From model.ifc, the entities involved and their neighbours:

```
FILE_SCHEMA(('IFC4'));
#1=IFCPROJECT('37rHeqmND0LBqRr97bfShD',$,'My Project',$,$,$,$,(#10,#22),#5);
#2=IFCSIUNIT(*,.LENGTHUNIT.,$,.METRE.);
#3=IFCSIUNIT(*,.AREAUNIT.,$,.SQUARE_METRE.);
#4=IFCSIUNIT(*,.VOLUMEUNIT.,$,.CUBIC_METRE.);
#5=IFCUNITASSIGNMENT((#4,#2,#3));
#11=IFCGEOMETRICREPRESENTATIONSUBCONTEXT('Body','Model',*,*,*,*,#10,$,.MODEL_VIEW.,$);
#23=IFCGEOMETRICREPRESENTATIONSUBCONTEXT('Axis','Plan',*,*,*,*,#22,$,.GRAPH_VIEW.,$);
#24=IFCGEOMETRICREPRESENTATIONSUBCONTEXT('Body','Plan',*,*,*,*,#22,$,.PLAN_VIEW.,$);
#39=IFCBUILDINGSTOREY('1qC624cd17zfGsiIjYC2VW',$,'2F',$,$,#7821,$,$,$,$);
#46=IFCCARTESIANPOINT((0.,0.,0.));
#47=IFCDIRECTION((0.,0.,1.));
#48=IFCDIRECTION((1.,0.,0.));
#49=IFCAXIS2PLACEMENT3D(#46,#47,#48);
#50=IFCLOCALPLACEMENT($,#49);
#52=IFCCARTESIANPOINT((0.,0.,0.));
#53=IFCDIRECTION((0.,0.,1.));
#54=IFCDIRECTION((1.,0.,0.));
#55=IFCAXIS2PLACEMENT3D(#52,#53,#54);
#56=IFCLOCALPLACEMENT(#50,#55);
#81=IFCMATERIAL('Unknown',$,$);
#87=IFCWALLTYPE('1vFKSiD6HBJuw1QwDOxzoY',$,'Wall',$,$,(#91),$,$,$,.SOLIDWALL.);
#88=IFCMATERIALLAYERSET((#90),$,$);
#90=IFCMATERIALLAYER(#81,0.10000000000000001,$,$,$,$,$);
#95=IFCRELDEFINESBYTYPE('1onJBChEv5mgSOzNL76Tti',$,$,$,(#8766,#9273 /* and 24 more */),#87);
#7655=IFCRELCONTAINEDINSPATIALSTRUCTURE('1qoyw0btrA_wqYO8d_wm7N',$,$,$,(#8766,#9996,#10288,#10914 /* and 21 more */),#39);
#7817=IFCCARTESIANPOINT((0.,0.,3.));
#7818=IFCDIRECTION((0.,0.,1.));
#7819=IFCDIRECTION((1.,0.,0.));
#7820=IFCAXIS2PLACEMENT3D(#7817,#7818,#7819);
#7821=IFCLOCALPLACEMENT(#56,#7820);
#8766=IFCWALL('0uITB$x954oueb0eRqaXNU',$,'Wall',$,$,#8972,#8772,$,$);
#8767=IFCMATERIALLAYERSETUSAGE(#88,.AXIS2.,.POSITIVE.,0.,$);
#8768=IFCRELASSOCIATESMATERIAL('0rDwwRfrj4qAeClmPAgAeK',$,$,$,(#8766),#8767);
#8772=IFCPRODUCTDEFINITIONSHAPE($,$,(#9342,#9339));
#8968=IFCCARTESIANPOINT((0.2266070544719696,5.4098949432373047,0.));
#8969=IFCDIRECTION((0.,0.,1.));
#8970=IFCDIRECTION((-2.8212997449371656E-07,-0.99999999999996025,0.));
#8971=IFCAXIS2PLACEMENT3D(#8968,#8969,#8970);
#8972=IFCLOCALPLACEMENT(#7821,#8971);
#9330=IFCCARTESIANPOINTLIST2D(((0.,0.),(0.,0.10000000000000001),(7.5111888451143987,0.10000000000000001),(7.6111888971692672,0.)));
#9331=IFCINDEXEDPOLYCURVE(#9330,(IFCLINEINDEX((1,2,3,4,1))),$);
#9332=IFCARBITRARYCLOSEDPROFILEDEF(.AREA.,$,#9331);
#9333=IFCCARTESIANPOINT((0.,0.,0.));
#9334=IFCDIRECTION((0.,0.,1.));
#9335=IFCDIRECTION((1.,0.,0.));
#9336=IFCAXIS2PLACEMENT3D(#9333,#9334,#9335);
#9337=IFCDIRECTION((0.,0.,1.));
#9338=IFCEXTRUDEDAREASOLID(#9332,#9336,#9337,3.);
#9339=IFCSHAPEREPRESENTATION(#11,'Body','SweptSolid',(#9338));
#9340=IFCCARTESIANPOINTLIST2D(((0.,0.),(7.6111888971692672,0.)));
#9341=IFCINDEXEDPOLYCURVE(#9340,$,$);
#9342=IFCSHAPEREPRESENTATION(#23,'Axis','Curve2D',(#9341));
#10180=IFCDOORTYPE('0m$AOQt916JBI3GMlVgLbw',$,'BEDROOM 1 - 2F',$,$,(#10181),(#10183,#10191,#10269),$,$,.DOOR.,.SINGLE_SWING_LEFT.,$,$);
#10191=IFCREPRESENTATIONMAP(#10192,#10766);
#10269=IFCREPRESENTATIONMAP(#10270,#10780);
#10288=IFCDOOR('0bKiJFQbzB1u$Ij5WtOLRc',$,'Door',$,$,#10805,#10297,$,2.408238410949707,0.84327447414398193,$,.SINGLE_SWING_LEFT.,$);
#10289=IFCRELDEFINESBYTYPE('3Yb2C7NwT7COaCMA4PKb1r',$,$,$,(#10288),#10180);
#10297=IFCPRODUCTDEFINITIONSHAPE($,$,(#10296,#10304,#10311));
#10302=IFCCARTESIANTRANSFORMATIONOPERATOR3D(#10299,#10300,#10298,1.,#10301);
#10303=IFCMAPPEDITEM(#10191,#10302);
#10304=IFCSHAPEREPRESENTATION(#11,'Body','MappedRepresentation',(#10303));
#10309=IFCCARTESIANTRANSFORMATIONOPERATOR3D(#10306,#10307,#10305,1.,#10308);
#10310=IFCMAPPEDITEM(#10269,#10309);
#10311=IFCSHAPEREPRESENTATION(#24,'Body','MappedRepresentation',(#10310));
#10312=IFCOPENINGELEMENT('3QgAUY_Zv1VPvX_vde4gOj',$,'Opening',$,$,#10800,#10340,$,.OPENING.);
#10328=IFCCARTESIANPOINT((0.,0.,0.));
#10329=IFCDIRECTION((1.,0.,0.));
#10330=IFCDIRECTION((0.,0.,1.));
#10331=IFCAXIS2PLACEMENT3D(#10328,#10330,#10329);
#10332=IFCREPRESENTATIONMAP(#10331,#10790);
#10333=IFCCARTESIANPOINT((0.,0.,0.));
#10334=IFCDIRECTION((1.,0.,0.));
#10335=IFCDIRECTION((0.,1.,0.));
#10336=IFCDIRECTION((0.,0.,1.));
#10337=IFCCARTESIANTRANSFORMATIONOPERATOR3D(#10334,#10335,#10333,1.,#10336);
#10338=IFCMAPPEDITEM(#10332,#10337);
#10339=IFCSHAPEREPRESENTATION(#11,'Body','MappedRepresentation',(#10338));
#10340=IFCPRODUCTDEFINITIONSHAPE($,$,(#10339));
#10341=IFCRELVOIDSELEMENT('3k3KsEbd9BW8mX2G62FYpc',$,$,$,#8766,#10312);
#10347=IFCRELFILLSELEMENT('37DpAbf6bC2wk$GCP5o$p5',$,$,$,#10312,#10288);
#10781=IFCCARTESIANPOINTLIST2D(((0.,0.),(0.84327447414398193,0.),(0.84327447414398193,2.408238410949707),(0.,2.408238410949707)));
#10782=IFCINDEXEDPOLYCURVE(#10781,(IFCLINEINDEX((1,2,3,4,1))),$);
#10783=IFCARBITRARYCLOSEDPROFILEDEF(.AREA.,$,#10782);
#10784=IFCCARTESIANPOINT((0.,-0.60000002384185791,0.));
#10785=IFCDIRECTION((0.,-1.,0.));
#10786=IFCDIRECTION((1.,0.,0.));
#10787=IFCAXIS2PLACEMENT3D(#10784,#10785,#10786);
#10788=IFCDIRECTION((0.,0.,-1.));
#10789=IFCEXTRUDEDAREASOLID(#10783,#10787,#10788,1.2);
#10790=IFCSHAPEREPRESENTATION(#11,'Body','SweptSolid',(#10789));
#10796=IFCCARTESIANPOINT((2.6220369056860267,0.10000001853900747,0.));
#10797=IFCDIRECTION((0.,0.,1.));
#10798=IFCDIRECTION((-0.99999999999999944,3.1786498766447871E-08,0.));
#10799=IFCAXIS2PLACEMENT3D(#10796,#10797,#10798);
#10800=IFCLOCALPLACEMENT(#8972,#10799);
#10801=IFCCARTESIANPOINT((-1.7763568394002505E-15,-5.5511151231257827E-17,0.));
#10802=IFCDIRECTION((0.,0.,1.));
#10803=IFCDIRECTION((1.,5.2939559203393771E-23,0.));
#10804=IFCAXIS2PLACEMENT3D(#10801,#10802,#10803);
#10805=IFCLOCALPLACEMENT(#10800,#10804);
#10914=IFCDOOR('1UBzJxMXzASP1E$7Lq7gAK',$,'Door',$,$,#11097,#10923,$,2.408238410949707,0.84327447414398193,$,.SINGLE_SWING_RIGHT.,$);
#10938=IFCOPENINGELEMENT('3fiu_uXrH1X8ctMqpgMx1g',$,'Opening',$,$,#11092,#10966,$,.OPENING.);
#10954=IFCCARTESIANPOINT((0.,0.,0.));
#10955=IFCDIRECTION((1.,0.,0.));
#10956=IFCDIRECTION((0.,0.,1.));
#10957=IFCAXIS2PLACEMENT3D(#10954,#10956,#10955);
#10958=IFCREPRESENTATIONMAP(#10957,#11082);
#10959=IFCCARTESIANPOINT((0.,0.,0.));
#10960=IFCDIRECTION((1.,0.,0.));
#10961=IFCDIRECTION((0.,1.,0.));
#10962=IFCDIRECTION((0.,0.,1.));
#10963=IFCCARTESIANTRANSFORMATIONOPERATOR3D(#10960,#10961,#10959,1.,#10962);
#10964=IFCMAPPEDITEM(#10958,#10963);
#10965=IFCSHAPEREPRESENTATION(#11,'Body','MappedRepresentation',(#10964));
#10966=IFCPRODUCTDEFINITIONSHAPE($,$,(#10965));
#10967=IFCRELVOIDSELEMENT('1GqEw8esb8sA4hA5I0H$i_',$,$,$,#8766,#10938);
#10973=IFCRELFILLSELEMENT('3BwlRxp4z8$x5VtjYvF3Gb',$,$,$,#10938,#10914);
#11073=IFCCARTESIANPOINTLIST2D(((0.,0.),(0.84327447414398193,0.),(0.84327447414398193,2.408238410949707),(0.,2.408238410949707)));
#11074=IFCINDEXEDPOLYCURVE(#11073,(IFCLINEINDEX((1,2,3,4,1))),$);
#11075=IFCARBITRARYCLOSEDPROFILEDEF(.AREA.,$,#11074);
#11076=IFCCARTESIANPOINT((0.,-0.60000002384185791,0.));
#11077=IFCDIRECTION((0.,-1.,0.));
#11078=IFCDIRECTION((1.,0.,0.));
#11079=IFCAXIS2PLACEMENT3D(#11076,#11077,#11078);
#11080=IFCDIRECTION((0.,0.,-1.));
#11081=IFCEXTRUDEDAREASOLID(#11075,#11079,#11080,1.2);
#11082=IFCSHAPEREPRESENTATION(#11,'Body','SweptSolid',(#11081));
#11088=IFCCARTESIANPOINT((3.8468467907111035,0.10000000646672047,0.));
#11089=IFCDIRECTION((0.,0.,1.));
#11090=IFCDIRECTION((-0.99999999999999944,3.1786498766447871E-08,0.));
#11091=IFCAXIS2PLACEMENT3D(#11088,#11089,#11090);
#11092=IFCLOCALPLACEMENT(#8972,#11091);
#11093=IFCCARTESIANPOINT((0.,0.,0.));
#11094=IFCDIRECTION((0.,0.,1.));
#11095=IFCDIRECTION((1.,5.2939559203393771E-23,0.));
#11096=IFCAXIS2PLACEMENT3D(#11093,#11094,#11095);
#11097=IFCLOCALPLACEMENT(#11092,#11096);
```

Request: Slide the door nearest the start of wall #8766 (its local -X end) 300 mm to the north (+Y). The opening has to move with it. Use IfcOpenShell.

```python
import ifcopenshell
import ifcopenshell.api.geometry
import ifcopenshell.util.placement

model = ifcopenshell.open("model.ifc")

door = model.by_guid("0bKiJFQbzB1u$Ij5WtOLRc")
opening = door.FillsVoids[0].RelatingOpeningElement
wall = opening.VoidsElements[0].RelatingBuildingElement

wall_matrix = ifcopenshell.util.placement.get_local_placement(wall.ObjectPlacement)
shift = wall_matrix[:3, 0] * -0.3
before = ifcopenshell.util.placement.get_local_placement(door.ObjectPlacement)[:3, 3].copy()

# The door is placed relative to its opening, so it follows when the opening moves.
matrix = ifcopenshell.util.placement.get_local_placement(opening.ObjectPlacement)
matrix[:3, 3] += shift
ifcopenshell.api.geometry.edit_object_placement(
    model, product=opening, matrix=matrix, is_si=False, should_transform_children=True
)

after = ifcopenshell.util.placement.get_local_placement(door.ObjectPlacement)[:3, 3]
print("door moved by", (after - before).round(3) + 0.0)

model.write("model_edited.ifc")
```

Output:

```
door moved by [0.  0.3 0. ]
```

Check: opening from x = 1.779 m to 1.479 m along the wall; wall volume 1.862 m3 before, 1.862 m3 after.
